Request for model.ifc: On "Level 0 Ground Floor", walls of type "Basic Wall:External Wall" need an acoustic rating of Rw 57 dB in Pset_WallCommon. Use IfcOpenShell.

First a look at what the model holds.

```python
import ifcopenshell
import ifcopenshell.util.element

model = ifcopenshell.open("model.ifc")
print(model.schema)
storey = next(s for s in model.by_type("IfcBuildingStorey") if s.Name == "Level 0 Ground Floor")
walls = [e for e in ifcopenshell.util.element.get_decomposition(storey) if e.is_a("IfcWall")]
seen = {}
for e in walls:
    element_type = ifcopenshell.util.element.get_type(e)
    key = (element_type.Name if element_type != e and element_type else None, ifcopenshell.util.element.get_pset(e, "Pset_WallCommon", "AcousticRating"))
    seen[key] = seen.get(key, 0) + 1
for (name, value), count in sorted(seen.items(), key=str):
    print(count, "x", name, "|", value)
```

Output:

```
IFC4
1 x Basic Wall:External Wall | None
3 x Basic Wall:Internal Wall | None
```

```python
import ifcopenshell
import ifcopenshell.api.pset
import ifcopenshell.util.element

model = ifcopenshell.open("model.ifc")

storey = next(s for s in model.by_type("IfcBuildingStorey") if s.Name == "Level 0 Ground Floor")
walls = [e for e in ifcopenshell.util.element.get_decomposition(storey) if e.is_a("IfcWall")]

count = 0
for e in walls:
    element_type = ifcopenshell.util.element.get_type(e)
    if element_type in (None, e) or element_type.Name != "Basic Wall:External Wall":
        continue
    # add_pset returns the element's existing set when there is one.
    pset = ifcopenshell.api.pset.add_pset(model, product=e, name="Pset_WallCommon")
    ifcopenshell.api.pset.edit_pset(model, pset=pset, properties={"AcousticRating": "Rw 57 dB"})
    count += 1

print(count, "walls updated")

model.write("model_v2.ifc")
```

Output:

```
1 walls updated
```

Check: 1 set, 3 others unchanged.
